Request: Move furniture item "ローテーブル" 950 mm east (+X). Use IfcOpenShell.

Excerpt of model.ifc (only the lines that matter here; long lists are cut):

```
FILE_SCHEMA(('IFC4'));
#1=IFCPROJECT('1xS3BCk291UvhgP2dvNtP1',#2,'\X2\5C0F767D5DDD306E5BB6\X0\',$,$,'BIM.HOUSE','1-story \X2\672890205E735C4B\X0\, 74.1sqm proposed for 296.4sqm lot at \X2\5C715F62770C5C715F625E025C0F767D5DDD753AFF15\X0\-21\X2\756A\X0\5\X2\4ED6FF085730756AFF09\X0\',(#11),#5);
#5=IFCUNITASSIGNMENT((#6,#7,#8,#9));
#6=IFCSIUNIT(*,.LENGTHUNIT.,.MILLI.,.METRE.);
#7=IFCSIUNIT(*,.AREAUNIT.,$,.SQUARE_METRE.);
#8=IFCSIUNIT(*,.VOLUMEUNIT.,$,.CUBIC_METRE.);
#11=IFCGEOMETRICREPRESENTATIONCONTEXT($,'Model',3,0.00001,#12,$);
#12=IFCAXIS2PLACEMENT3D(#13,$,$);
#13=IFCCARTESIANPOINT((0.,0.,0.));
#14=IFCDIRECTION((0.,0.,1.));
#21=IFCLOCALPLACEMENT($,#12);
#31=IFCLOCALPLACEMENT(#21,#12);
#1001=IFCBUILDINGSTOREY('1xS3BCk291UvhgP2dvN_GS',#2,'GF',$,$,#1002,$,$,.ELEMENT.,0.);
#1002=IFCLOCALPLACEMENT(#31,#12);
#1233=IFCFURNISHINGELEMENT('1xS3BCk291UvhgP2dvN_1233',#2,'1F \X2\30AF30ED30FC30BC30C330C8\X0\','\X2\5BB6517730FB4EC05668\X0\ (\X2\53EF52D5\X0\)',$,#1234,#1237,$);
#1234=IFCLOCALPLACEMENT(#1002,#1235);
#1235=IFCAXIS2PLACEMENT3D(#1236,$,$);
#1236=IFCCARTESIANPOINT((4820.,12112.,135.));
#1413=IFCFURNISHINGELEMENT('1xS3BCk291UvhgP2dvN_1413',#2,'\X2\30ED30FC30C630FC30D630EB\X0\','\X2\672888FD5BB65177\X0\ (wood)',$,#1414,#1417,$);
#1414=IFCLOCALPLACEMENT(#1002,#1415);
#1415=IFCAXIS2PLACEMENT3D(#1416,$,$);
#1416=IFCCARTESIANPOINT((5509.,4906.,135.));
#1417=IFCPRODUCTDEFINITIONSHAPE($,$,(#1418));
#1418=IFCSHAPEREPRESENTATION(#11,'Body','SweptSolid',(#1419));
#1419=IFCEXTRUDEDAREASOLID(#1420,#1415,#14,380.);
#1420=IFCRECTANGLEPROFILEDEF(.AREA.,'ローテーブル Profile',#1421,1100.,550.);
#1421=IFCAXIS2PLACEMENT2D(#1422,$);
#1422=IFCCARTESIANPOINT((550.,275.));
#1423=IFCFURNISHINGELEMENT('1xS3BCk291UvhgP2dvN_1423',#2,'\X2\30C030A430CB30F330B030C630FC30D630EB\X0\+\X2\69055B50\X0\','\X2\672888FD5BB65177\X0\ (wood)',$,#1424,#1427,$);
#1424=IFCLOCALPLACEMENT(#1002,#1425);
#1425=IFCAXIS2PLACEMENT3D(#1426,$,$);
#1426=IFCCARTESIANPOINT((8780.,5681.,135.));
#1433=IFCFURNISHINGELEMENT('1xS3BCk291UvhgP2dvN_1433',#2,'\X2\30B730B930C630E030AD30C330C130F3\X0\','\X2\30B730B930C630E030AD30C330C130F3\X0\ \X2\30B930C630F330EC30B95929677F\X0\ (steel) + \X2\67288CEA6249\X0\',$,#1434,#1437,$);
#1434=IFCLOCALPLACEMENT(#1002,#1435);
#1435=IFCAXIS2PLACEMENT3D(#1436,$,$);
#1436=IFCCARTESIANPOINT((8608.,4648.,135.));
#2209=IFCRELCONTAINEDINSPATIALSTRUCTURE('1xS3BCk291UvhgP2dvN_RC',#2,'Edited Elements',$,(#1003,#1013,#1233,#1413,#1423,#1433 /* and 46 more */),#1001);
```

```python
import ifcopenshell
import ifcopenshell.api.geometry
import ifcopenshell.util.placement
import ifcopenshell.util.unit

model = ifcopenshell.open("model.ifc")
unit_scale = ifcopenshell.util.unit.calculate_unit_scale(model)

item = model.by_id(1413)
matrix = ifcopenshell.util.placement.get_local_placement(item.ObjectPlacement)
matrix[0, 3] += 0.95 / unit_scale
ifcopenshell.api.geometry.edit_object_placement(model, product=item, matrix=matrix, is_si=False)

print(ifcopenshell.util.placement.get_local_placement(item.ObjectPlacement).round(3) + 0.0)

model.write("model_edited.ifc")
```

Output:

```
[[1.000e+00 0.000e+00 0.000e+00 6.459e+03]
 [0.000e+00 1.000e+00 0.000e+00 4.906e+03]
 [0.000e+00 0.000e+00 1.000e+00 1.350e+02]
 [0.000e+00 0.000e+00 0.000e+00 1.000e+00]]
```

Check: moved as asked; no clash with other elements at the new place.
